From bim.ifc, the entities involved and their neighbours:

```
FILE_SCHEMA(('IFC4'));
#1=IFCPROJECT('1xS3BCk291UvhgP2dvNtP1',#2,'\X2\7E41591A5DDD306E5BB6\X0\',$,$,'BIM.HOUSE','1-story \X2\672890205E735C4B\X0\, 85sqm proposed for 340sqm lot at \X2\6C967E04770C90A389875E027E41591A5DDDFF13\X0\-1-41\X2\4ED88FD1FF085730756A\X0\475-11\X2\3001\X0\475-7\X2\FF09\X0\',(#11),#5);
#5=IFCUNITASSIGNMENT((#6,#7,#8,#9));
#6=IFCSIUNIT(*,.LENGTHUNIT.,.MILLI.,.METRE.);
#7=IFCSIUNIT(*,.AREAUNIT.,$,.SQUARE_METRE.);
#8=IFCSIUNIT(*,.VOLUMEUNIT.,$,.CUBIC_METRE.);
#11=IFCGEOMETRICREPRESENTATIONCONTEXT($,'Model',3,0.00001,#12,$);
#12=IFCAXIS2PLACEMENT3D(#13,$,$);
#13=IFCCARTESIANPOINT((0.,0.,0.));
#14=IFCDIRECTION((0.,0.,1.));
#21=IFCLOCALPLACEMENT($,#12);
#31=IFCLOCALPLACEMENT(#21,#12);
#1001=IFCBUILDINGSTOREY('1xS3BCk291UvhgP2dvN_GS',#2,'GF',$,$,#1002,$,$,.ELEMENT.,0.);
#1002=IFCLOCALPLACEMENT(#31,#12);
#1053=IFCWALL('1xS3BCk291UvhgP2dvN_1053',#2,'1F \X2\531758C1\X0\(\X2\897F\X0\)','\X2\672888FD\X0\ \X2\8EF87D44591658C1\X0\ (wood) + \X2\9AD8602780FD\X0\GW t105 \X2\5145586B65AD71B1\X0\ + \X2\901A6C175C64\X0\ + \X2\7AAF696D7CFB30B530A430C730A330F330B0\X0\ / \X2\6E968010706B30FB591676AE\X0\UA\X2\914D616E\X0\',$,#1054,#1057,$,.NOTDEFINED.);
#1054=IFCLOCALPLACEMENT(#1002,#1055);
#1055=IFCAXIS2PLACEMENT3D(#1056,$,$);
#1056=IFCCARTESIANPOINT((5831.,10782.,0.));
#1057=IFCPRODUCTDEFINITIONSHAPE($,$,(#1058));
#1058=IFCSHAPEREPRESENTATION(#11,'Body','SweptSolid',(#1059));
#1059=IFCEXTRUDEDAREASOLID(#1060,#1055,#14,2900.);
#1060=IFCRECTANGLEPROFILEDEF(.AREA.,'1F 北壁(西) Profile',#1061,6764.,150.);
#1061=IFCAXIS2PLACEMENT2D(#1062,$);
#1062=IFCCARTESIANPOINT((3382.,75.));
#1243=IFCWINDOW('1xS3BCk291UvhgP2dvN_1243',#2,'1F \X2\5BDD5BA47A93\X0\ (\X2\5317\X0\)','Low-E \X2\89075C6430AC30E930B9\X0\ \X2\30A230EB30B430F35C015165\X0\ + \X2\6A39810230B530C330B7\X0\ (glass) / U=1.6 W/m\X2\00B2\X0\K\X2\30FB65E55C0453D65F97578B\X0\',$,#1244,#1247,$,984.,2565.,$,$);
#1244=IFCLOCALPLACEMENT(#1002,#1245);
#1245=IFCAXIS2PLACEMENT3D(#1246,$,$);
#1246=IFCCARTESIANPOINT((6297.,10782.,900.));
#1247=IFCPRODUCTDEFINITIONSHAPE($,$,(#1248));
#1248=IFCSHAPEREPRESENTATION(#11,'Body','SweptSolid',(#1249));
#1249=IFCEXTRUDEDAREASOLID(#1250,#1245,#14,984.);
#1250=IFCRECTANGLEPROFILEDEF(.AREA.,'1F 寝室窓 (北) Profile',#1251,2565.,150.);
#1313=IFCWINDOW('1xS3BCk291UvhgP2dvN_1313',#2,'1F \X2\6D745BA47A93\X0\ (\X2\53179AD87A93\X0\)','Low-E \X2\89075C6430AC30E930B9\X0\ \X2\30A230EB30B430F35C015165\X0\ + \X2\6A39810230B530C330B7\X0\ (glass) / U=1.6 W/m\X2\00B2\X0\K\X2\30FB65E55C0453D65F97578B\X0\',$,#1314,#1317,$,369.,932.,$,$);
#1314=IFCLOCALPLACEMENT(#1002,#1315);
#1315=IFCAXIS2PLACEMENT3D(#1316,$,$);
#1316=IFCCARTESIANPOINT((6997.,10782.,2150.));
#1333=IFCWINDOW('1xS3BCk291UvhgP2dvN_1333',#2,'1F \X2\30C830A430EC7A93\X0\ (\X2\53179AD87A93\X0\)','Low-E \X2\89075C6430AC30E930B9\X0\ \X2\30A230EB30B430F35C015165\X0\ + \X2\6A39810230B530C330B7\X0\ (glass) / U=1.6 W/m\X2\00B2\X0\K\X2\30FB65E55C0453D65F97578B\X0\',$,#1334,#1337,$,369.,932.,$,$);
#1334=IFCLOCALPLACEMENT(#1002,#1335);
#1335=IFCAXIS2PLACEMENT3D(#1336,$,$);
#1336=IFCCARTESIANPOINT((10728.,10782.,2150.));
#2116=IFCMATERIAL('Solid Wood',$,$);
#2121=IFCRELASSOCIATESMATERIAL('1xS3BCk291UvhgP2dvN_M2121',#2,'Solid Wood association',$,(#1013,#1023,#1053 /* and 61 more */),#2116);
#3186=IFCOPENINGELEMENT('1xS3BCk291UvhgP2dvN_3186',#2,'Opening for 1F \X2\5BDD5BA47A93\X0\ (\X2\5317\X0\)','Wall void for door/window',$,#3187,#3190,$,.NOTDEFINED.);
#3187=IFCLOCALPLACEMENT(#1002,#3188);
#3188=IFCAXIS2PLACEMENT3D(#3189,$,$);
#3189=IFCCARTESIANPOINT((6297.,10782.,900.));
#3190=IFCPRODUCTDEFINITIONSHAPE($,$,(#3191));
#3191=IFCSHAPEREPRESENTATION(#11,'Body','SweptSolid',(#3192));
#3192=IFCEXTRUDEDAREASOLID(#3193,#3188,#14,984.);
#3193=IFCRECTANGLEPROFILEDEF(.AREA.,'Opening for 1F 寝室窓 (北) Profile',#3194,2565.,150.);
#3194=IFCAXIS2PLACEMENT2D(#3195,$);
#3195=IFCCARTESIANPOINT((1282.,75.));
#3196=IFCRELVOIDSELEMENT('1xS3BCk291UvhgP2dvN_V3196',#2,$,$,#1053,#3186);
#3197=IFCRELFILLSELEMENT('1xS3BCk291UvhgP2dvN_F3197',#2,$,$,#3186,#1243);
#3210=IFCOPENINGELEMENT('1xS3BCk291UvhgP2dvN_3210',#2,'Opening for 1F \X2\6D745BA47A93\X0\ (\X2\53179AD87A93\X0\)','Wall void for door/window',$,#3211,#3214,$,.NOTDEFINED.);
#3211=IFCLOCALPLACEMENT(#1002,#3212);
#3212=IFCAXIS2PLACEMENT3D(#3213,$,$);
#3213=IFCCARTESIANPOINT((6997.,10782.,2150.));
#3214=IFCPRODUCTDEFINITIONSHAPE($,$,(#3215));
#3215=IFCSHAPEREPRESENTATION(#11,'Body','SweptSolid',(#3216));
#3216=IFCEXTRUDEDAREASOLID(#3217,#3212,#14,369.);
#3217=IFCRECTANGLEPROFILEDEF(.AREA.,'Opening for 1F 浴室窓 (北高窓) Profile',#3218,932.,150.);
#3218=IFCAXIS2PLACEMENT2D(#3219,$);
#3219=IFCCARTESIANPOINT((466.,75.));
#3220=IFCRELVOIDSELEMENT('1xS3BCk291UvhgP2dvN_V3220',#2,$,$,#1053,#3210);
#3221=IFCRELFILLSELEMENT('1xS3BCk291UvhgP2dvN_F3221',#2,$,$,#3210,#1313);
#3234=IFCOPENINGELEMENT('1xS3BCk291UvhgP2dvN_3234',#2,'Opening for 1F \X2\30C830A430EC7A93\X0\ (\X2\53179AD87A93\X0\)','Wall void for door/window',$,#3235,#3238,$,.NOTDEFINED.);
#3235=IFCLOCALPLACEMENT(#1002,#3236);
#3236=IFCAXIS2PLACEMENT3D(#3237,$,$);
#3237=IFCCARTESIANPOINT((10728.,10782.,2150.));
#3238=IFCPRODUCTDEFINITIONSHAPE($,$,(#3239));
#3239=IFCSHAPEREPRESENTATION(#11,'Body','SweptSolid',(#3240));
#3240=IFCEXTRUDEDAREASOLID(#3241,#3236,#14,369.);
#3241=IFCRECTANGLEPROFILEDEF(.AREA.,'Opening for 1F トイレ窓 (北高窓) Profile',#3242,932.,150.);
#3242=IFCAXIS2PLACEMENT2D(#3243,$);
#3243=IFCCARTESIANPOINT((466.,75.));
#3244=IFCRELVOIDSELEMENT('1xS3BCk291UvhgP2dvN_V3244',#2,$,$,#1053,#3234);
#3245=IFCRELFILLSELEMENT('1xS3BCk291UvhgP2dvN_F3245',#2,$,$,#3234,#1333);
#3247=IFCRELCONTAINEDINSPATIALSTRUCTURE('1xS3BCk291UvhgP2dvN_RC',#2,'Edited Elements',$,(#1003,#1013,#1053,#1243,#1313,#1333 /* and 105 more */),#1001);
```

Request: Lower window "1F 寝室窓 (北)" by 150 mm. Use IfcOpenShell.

```python
import numpy as np
import ifcopenshell
import ifcopenshell.api.geometry
import ifcopenshell.util.placement
import ifcopenshell.util.unit

model = ifcopenshell.open("bim.ifc")
unit_scale = ifcopenshell.util.unit.calculate_unit_scale(model)

window = model.by_id(1243)
opening = window.FillsVoids[0].RelatingOpeningElement
dz = -0.15 / unit_scale

shift = np.array([0.0, 0.0, dz])
# The window is not placed relative to its opening, so move both.
for product in (opening, window):
    matrix = ifcopenshell.util.placement.get_local_placement(product.ObjectPlacement)
    matrix[:3, 3] += shift
    ifcopenshell.api.geometry.edit_object_placement(model, product=product, matrix=matrix, is_si=False)

print(f"moved by {dz * unit_scale:+.3f} m")

model.write("bim_updated.ifc")
```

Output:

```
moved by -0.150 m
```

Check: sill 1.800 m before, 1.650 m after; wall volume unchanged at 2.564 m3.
